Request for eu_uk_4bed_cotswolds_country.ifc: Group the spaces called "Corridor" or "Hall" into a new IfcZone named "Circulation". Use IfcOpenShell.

First a look at what the model holds.

```python
import ifcopenshell

model = ifcopenshell.open("eu_uk_4bed_cotswolds_country.ifc")
print(model.schema)
seen = {}
for space in model.by_type("IfcSpace"):
    seen[space.LongName] = seen.get(space.LongName, 0) + 1
for name, count in sorted(seen.items(), key=str):
    print(count, "x", name)
print("zones:", [z.Name for z in model.by_type("IfcZone")][:20])
```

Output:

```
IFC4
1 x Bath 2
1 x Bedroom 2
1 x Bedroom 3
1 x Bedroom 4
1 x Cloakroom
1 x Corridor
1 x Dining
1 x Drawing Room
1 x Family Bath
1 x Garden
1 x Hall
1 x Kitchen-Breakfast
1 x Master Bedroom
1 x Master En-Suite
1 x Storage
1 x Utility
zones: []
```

```python
import ifcopenshell
import ifcopenshell.api.group
import ifcopenshell.api.root

model = ifcopenshell.open("eu_uk_4bed_cotswolds_country.ifc")

names = {"Corridor", "Hall"}
spaces = [s for s in model.by_type("IfcSpace") if s.LongName in names]

zone = ifcopenshell.api.root.create_entity(model, ifc_class="IfcZone", name="Circulation")
ifcopenshell.api.group.assign_group(model, products=spaces, group=zone)
print(len(spaces), "spaces in", zone.Name)

model.write("eu_uk_4bed_cotswolds_country_rev.ifc")
```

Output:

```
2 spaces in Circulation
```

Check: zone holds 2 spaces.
